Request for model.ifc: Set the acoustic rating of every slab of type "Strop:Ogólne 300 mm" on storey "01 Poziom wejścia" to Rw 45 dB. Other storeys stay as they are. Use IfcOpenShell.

First a look at what the model holds.

```python
import ifcopenshell
import ifcopenshell.util.element

model = ifcopenshell.open("model.ifc")
print(model.schema)
storey = next(s for s in model.by_type("IfcBuildingStorey") if s.Name == "01 Poziom wejścia")
slabs = [e for e in ifcopenshell.util.element.get_decomposition(storey) if e.is_a("IfcSlab")]
seen = {}
for e in slabs:
    element_type = ifcopenshell.util.element.get_type(e)
    key = (element_type.Name if element_type != e and element_type else None, ifcopenshell.util.element.get_pset(e, "Pset_SlabCommon", "AcousticRating"))
    seen[key] = seen.get(key, 0) + 1
for (name, value), count in sorted(seen.items(), key=str):
    print(count, "x", name, "|", value)
```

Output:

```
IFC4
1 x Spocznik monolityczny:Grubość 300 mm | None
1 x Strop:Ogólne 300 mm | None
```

```python
import ifcopenshell
import ifcopenshell.api.pset
import ifcopenshell.util.element

model = ifcopenshell.open("model.ifc")

storey = next(s for s in model.by_type("IfcBuildingStorey") if s.Name == "01 Poziom wejścia")
slabs = [e for e in ifcopenshell.util.element.get_decomposition(storey) if e.is_a("IfcSlab")]

count = 0
for e in slabs:
    element_type = ifcopenshell.util.element.get_type(e)
    if element_type in (None, e) or element_type.Name != "Strop:Ogólne 300 mm":
        continue
    # add_pset returns the element's existing set when there is one.
    pset = ifcopenshell.api.pset.add_pset(model, product=e, name="Pset_SlabCommon")
    ifcopenshell.api.pset.edit_pset(model, pset=pset, properties={"AcousticRating": "Rw 45 dB"})
    count += 1

print(count, "slabs updated")

model.write("model_v2.ifc")
```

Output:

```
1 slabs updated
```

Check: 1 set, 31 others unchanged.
